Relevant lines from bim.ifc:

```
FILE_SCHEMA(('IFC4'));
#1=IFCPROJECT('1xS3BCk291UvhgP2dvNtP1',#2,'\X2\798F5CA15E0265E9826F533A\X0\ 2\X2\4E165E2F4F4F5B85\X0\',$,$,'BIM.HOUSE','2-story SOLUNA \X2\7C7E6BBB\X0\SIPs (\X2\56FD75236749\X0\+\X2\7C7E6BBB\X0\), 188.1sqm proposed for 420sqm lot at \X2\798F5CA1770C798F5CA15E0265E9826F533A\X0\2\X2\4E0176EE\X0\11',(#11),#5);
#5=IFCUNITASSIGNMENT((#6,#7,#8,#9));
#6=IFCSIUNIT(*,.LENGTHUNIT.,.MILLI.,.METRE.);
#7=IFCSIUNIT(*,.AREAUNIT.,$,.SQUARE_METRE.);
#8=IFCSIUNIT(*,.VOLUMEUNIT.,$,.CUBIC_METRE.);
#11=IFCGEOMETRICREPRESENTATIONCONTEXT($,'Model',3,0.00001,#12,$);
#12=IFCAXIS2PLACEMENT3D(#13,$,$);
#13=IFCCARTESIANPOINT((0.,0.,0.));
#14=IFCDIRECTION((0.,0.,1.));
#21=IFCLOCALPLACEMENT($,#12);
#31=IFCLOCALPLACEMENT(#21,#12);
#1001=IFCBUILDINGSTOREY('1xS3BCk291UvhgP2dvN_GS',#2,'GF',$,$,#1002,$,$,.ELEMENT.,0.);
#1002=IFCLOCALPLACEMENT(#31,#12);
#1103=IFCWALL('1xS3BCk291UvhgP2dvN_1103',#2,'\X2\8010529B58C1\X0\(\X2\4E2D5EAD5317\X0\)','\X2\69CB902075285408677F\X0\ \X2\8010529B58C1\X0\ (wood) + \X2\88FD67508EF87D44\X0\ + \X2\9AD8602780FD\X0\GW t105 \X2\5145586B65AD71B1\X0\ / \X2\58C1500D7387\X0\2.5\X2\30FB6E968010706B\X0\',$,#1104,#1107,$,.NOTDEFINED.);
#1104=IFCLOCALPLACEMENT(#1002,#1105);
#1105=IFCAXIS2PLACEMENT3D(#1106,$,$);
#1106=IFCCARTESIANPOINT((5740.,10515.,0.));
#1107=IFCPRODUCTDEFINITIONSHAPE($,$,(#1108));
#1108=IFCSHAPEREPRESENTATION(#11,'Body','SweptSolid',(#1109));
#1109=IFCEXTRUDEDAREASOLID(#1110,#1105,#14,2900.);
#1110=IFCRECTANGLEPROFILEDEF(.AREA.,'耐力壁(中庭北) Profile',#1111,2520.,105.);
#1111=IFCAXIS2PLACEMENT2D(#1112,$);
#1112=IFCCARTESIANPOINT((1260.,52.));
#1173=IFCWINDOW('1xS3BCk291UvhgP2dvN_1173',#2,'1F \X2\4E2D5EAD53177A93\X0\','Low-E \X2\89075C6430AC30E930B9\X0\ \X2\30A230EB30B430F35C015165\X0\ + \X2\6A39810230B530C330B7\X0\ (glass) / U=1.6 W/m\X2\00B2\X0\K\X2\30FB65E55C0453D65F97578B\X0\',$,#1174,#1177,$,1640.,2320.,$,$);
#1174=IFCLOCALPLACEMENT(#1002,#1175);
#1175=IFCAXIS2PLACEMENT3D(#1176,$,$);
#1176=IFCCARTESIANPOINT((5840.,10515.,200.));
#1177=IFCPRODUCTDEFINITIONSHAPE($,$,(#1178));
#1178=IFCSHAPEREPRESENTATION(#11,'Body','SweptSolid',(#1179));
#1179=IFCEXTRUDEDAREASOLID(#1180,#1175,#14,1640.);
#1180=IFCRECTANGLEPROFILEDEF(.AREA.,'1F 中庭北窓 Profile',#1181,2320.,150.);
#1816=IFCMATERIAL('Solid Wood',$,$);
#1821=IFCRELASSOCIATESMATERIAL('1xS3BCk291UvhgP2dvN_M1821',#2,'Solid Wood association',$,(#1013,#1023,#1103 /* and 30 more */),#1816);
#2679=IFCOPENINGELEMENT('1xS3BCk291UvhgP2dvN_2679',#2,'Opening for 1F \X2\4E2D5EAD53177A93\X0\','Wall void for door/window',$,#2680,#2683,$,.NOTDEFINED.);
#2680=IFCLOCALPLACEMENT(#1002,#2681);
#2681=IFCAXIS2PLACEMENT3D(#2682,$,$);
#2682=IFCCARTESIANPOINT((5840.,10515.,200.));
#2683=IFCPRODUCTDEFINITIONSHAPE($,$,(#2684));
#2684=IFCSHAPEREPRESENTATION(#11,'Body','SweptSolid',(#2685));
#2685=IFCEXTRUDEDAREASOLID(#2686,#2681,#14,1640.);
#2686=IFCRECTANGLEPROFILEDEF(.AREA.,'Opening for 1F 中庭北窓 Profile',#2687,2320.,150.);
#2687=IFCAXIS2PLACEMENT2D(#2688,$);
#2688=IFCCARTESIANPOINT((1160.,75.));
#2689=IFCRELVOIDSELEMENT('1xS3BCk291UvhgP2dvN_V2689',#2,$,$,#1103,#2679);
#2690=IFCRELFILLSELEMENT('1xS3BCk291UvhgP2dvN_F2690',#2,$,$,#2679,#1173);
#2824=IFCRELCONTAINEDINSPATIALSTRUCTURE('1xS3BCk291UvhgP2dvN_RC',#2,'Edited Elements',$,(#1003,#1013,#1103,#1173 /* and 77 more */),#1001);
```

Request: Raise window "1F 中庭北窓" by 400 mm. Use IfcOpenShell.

```python
import numpy as np
import ifcopenshell
import ifcopenshell.api.geometry
import ifcopenshell.util.placement
import ifcopenshell.util.unit

model = ifcopenshell.open("bim.ifc")
unit_scale = ifcopenshell.util.unit.calculate_unit_scale(model)

window = model.by_guid("1xS3BCk291UvhgP2dvN_1173")
opening = window.FillsVoids[0].RelatingOpeningElement
dz = 0.4 / unit_scale

shift = np.array([0.0, 0.0, dz])
# The window is not placed relative to its opening, so move both.
for product in (opening, window):
    matrix = ifcopenshell.util.placement.get_local_placement(product.ObjectPlacement)
    matrix[:3, 3] += shift
    ifcopenshell.api.geometry.edit_object_placement(model, product=product, matrix=matrix, is_si=False)

print(f"moved by {dz * unit_scale:+.3f} m")

model.write("bim_v2.ifc")
```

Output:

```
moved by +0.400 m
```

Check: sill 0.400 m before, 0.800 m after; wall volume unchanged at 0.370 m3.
